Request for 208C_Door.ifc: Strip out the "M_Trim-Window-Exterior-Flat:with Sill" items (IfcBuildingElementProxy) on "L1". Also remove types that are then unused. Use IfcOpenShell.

First a look at what the model holds.

```python
import ifcopenshell
import ifcopenshell.util.element

model = ifcopenshell.open("208C_Door.ifc")
print(model.schema)
storey = next(s for s in model.by_type("IfcBuildingStorey") if s.Name == "L1")
proxies = [e for e in ifcopenshell.util.element.get_decomposition(storey) if e.is_a("IfcBuildingElementProxy")]
seen = {}
for e in proxies:
    element_type = ifcopenshell.util.element.get_type(e)
    name = element_type.Name if element_type not in (None, e) else None
    seen[name] = seen.get(name, 0) + 1
for name, count in sorted(seen.items(), key=str):
    print(count, "x", name)
```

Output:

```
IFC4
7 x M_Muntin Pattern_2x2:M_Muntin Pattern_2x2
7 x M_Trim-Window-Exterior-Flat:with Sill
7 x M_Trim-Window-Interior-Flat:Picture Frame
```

```python
import ifcopenshell
import ifcopenshell.api.root
import ifcopenshell.util.element

model = ifcopenshell.open("208C_Door.ifc")

storey = next(s for s in model.by_type("IfcBuildingStorey") if s.Name == "L1")
proxies = [e for e in ifcopenshell.util.element.get_decomposition(storey) if e.is_a("IfcBuildingElementProxy")]
targets = [e for e in proxies if (t := ifcopenshell.util.element.get_type(e)) not in (None, e) and t.Name == "M_Trim-Window-Exterior-Flat:with Sill"]
types = {ifcopenshell.util.element.get_type(e) for e in targets} - {None, *targets}

for e in targets:
    ifcopenshell.api.root.remove_product(model, product=e)
print(len(targets), "removed")

unused = [t for t in types if not ifcopenshell.util.element.get_types(t)]
for t in unused:
    ifcopenshell.api.root.remove_product(model, product=t)
print(len(unused), "unused types removed")

model.write("208C_Door_updated.ifc")
```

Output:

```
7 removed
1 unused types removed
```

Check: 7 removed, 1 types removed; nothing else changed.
